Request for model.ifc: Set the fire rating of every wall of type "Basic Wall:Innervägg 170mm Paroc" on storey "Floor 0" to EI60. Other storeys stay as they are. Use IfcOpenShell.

First a look at what the model holds.

```python
import ifcopenshell
import ifcopenshell.util.element

model = ifcopenshell.open("model.ifc")
print(model.schema)
storey = next(s for s in model.by_type("IfcBuildingStorey") if s.Name == "Floor 0")
walls = [e for e in ifcopenshell.util.element.get_decomposition(storey) if e.is_a("IfcWall")]
seen = {}
for e in walls:
    element_type = ifcopenshell.util.element.get_type(e)
    key = (element_type.Name if element_type != e and element_type else None, ifcopenshell.util.element.get_pset(e, "Pset_WallCommon", "FireRating"))
    seen[key] = seen.get(key, 0) + 1
for (name, value), count in sorted(seen.items(), key=str):
    print(count, "x", name, "|", value)
```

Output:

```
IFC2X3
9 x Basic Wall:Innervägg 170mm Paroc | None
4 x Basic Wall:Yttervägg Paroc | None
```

```python
import ifcopenshell
import ifcopenshell.api.pset
import ifcopenshell.util.element

model = ifcopenshell.open("model.ifc")

storey = next(s for s in model.by_type("IfcBuildingStorey") if s.Name == "Floor 0")
walls = [e for e in ifcopenshell.util.element.get_decomposition(storey) if e.is_a("IfcWall")]

count = 0
for e in walls:
    element_type = ifcopenshell.util.element.get_type(e)
    if element_type in (None, e) or element_type.Name != "Basic Wall:Innervägg 170mm Paroc":
        continue
    # add_pset returns the element's existing set when there is one.
    pset = ifcopenshell.api.pset.add_pset(model, product=e, name="Pset_WallCommon")
    ifcopenshell.api.pset.edit_pset(model, pset=pset, properties={"FireRating": "EI60"})
    count += 1

print(count, "walls updated")

model.write("model_rev.ifc")
```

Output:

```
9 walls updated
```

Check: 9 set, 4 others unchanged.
